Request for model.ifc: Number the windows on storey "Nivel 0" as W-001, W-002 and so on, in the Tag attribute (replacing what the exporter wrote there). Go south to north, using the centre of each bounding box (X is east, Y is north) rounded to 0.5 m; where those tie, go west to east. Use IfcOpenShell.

First a look at what the model holds.

```python
import ifcopenshell
import ifcopenshell.util.element
import ifcopenshell.util.placement

model = ifcopenshell.open("model.ifc")
print(model.schema)
storey = next(s for s in model.by_type("IfcBuildingStorey") if s.Name == "Nivel 0")
windows = [e for e in ifcopenshell.util.element.get_decomposition(storey) if e.is_a("IfcWindow")]
for e in sorted(windows, key=lambda e: e.id()):
    origin = ifcopenshell.util.placement.get_local_placement(e.ObjectPlacement)[:3, 3]
    print(e.id(), e.Tag, e.Name, origin.round(2) + 0.0, sep=" | ")
```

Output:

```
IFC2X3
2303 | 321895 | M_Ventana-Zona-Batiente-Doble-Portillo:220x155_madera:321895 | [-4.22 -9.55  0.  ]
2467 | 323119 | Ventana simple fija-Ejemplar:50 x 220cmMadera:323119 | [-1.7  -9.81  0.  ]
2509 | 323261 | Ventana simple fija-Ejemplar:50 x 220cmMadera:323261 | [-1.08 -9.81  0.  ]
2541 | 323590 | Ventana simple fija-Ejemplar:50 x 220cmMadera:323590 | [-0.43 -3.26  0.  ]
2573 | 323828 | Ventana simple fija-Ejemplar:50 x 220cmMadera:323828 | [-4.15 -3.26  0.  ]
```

```python
import ifcopenshell
import ifcopenshell.geom
import ifcopenshell.util.element
import ifcopenshell.util.shape

model = ifcopenshell.open("model.ifc")
settings = ifcopenshell.geom.settings()
settings.set("use-world-coords", True)


def centre(element):
    shape = ifcopenshell.geom.create_shape(settings, element)
    return ifcopenshell.util.shape.get_bbox_centroid(shape.geometry)


storey = next(s for s in model.by_type("IfcBuildingStorey") if s.Name == "Nivel 0")
windows = [e for e in ifcopenshell.util.element.get_decomposition(storey) if e.is_a("IfcWindow")]

# Insertion points can sit at a corner or the storey origin, so sort by the geometry (in metres).
centres = {e: centre(e) for e in windows}
windows.sort(key=lambda e: (round(centres[e][1] / 0.5), centres[e][0]))

for i, e in enumerate(windows, start=1):
    number = f"W-0{i:02d}"
    e.Tag = number
    print(e.id(), number)

model.write("model_edited.ifc")
```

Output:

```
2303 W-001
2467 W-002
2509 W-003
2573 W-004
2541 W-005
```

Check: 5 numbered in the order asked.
